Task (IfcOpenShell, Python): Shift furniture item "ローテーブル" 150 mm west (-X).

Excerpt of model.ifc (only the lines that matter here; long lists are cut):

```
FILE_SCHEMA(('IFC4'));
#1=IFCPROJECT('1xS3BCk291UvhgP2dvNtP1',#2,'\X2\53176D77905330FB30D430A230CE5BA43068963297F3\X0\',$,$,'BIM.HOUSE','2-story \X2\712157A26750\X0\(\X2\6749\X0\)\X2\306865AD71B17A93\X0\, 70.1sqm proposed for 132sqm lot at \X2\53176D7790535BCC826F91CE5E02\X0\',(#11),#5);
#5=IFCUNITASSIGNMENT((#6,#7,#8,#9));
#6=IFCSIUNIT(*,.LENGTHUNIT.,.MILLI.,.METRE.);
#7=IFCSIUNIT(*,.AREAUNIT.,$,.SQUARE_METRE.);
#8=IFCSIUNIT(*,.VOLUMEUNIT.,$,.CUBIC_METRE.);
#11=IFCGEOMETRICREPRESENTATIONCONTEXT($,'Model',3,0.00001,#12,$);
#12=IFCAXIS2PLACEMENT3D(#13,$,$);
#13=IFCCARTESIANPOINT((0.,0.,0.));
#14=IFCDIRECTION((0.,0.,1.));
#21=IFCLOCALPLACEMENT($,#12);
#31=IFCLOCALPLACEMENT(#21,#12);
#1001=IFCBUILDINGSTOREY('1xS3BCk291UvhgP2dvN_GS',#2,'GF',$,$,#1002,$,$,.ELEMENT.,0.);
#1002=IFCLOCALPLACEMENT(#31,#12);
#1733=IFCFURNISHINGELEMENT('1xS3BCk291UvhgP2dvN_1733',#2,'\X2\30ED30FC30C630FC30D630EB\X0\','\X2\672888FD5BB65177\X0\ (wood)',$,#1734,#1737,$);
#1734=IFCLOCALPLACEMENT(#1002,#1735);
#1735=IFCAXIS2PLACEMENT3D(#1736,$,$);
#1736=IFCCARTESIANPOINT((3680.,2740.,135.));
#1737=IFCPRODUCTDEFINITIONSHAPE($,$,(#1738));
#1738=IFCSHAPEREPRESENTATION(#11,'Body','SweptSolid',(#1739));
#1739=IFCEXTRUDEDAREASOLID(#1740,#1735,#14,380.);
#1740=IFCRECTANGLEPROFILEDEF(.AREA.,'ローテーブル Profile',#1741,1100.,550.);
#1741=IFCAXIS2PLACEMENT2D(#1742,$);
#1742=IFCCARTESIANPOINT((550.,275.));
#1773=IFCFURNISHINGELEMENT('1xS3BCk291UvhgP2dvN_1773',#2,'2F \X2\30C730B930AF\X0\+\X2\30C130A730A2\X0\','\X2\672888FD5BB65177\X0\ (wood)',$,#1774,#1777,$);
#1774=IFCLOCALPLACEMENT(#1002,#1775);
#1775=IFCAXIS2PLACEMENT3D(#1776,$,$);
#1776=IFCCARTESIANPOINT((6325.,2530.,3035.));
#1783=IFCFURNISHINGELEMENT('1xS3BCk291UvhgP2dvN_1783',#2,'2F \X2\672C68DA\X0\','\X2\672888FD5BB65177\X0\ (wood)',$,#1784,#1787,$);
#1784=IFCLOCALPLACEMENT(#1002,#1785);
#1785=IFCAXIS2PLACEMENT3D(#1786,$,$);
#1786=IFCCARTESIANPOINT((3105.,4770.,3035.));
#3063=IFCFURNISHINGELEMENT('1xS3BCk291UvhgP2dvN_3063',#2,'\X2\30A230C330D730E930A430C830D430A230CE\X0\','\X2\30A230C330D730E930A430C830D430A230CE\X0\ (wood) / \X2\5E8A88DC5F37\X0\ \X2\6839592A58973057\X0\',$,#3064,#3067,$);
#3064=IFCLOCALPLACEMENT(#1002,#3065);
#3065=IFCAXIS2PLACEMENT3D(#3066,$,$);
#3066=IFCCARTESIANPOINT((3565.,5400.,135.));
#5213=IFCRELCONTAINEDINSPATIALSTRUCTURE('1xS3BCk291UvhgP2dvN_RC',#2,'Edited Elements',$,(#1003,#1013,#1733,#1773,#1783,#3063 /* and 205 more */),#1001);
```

```python
import ifcopenshell
import ifcopenshell.api.geometry
import ifcopenshell.util.placement
import ifcopenshell.util.unit

model = ifcopenshell.open("model.ifc")
unit_scale = ifcopenshell.util.unit.calculate_unit_scale(model)

item = model.by_id(1733)
matrix = ifcopenshell.util.placement.get_local_placement(item.ObjectPlacement)
matrix[0, 3] -= 0.15 / unit_scale
ifcopenshell.api.geometry.edit_object_placement(model, product=item, matrix=matrix, is_si=False)

print(ifcopenshell.util.placement.get_local_placement(item.ObjectPlacement).round(3) + 0.0)

model.write("model-out.ifc")
```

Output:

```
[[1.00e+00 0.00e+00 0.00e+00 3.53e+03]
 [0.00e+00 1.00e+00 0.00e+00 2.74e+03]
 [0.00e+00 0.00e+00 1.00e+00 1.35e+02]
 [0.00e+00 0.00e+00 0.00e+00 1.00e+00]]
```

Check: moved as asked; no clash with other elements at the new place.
